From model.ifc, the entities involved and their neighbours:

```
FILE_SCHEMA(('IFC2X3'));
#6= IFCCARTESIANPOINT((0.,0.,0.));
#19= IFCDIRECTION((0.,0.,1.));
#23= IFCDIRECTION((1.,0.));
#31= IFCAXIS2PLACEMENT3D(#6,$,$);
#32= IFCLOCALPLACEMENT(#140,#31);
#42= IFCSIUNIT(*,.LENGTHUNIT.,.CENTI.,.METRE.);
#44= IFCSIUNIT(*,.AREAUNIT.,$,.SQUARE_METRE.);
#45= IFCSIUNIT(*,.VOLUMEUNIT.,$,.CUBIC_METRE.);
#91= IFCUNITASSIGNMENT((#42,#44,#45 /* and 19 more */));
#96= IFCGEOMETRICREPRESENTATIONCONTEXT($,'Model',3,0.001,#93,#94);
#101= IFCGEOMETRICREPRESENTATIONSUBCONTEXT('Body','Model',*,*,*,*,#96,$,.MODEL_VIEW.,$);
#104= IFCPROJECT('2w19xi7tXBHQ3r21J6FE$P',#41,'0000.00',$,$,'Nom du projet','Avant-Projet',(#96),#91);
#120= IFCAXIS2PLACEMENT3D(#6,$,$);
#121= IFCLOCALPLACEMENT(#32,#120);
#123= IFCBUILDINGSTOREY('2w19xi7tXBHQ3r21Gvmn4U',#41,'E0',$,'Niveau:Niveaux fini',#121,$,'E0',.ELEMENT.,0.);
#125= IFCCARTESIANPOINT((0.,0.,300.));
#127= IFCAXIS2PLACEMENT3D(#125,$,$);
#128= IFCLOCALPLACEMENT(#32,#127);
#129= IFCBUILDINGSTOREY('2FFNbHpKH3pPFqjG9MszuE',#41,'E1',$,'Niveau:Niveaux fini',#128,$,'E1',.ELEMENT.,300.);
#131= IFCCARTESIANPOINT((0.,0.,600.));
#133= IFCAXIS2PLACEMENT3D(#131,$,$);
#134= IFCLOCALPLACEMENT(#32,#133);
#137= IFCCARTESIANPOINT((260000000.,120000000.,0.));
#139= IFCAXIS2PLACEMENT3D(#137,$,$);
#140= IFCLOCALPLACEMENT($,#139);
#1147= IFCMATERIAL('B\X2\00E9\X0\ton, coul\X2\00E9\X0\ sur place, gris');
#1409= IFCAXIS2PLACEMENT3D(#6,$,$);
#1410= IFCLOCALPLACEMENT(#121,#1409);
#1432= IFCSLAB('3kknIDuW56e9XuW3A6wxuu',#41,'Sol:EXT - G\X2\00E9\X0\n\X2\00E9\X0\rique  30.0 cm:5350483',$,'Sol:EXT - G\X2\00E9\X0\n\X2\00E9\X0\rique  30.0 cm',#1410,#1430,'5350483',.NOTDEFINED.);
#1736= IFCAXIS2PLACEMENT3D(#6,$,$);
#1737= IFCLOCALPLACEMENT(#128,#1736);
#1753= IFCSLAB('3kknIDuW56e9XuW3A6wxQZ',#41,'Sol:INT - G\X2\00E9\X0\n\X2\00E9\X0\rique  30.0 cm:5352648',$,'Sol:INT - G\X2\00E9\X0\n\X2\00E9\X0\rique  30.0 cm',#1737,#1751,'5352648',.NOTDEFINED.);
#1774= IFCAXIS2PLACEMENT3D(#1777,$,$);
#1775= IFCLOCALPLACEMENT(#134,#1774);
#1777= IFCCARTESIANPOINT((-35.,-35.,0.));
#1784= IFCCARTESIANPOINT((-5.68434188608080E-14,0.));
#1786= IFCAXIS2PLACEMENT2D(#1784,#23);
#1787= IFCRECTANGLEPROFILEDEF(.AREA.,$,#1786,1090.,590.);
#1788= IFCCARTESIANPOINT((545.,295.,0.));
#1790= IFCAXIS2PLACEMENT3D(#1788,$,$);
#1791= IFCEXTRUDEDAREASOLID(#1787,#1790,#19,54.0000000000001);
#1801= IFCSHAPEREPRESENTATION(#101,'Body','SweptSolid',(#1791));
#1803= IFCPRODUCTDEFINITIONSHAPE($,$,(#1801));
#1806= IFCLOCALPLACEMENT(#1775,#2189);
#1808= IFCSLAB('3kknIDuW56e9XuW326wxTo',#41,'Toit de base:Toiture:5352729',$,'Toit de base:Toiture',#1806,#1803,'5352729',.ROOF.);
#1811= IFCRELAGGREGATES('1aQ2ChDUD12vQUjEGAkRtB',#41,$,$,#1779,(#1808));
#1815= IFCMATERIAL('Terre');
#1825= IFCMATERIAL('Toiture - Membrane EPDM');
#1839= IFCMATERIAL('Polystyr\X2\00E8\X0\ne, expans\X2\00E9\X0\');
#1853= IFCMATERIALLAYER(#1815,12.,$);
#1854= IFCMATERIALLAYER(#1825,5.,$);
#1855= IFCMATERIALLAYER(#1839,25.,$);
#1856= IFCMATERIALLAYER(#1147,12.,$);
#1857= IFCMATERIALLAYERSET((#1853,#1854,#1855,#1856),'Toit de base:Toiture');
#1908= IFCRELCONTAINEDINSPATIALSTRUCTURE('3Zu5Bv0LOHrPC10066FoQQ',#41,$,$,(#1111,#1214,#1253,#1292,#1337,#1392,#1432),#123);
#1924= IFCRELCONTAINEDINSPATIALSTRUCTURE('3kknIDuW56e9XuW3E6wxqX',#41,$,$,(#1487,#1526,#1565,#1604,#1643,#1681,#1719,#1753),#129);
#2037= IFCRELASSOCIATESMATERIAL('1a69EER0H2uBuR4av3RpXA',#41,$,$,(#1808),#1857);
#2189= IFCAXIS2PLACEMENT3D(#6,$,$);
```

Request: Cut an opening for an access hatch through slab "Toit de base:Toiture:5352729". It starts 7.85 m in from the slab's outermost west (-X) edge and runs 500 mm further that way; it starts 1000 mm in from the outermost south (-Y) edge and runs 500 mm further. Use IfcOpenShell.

```python
import numpy as np
import ifcopenshell
import ifcopenshell.api.feature
import ifcopenshell.api.geometry
import ifcopenshell.api.root
import ifcopenshell.geom
import ifcopenshell.util.placement
import ifcopenshell.util.representation
import ifcopenshell.util.shape
import ifcopenshell.util.unit

model = ifcopenshell.open("model.ifc")
unit_scale = ifcopenshell.util.unit.calculate_unit_scale(model)
settings = ifcopenshell.geom.settings()


def volume(element):
    """Net volume in cubic metres, openings subtracted."""
    shape = ifcopenshell.geom.create_shape(settings, element)
    return ifcopenshell.util.shape.get_volume(shape.geometry)


slab = model.by_guid("3kknIDuW56e9XuW326wxTo")
before = volume(slab)

# Extent in the slab's own axes, in metres. The edges named are its -X and -Y sides.
slab_shape = ifcopenshell.geom.create_shape(settings, slab)
vertices = ifcopenshell.util.shape.get_vertices(slab_shape.geometry)
x_min, y_min, bottom = vertices.min(axis=0)
top = vertices[:, 2].max()

opening = ifcopenshell.api.root.create_entity(model, ifc_class="IfcOpeningElement", name="Access hatch opening")
context = ifcopenshell.util.representation.get_context(model, "Model", "Body", "MODEL_VIEW")
width, depth = 0.5, 0.5
outline = [(0.0, 0.0), (width, 0.0), (width, depth), (0.0, depth), (0.0, 0.0)]
# Overshoot both faces by 50 mm so the cut is clean.
shape = ifcopenshell.api.geometry.add_slab_representation(
    model, context=context, depth=top - bottom + 0.1, polyline=outline
)
ifcopenshell.api.geometry.assign_representation(model, product=opening, representation=shape)

matrix = ifcopenshell.util.placement.get_local_placement(slab.ObjectPlacement)
matrix[:, 3] = matrix @ np.append(np.array([x_min + 7.85, y_min + 1, bottom - 0.05]) / unit_scale, 1.0)
ifcopenshell.api.geometry.edit_object_placement(model, product=opening, matrix=matrix, is_si=False)
ifcopenshell.api.feature.add_feature(model, feature=opening, element=slab)

after = volume(slab)

print(f"slab volume {before:.3f} -> {after:.3f} m3")

model.write("model_updated.ifc")
```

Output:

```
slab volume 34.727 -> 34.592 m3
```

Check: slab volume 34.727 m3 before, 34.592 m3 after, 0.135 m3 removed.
